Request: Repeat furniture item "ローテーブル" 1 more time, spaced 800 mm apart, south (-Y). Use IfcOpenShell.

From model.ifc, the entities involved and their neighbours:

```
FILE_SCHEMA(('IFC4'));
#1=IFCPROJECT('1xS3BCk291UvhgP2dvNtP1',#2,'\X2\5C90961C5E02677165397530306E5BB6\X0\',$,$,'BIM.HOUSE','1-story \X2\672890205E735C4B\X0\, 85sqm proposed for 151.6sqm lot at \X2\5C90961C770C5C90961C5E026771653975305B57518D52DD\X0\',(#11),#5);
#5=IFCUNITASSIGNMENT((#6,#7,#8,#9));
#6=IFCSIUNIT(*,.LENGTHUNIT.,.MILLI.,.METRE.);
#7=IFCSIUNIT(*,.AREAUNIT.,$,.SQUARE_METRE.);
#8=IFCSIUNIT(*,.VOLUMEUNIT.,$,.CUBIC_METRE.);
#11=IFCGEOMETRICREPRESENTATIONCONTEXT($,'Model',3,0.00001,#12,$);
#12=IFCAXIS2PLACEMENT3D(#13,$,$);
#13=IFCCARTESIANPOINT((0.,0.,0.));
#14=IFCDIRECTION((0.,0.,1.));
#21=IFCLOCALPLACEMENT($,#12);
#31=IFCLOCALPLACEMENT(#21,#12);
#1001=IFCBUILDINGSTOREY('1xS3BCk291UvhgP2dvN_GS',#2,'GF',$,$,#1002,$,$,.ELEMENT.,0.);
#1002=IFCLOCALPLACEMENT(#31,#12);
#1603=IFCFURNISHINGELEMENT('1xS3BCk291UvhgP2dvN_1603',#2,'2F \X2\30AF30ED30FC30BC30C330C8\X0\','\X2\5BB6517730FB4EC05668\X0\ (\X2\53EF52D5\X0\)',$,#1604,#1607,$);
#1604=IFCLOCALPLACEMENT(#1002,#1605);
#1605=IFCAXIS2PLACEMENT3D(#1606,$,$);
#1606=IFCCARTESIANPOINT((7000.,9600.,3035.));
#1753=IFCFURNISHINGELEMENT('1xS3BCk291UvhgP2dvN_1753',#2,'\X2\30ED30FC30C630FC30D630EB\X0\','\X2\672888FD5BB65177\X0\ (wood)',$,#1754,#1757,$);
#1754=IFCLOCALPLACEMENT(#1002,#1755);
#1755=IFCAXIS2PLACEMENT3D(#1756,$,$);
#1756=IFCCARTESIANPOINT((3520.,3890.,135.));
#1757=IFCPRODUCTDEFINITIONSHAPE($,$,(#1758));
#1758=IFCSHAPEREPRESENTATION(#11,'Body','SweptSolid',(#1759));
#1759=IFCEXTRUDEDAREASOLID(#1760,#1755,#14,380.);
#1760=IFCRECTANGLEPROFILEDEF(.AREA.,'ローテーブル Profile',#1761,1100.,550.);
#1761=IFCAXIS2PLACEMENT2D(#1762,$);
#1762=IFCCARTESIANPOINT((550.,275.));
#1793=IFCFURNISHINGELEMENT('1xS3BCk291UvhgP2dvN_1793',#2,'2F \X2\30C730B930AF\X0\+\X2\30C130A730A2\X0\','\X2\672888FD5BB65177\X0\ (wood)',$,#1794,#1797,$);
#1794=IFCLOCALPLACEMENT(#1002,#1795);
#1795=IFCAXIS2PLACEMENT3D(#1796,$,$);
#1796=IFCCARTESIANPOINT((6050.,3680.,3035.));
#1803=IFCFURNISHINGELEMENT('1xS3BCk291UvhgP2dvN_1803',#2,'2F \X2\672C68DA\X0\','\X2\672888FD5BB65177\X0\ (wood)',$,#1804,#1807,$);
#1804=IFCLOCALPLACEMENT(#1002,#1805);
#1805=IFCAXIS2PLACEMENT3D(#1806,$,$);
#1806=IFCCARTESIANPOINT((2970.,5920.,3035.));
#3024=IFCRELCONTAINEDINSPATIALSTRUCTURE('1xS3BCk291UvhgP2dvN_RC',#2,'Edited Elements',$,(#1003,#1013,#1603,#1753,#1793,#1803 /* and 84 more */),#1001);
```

```python
import numpy as np
import ifcopenshell
import ifcopenshell.api.geometry
import ifcopenshell.api.root
import ifcopenshell.util.element
import ifcopenshell.util.placement
import ifcopenshell.util.unit

model = ifcopenshell.open("model.ifc")
unit_scale = ifcopenshell.util.unit.calculate_unit_scale(model)


def reuse_history(source, copy):
    """copy_class also copies each property set's owner history, people and application; keep the originals."""
    for rel in copy.IsDefinedBy:
        if rel.is_a("IfcRelDefinesByProperties") and (history := rel.RelatingPropertyDefinition.OwnerHistory):
            rel.RelatingPropertyDefinition.OwnerHistory = source.OwnerHistory
            ifcopenshell.util.element.remove_deep2(model, history)


source = model.by_id(1753)
base = ifcopenshell.util.placement.get_local_placement(source.ObjectPlacement)
step = np.array([0.0, -1.0, 0.0]) * 0.8 / unit_scale

for i in range(1, 2):
    copy = ifcopenshell.api.root.copy_class(model, product=source)
    copy.Representation = ifcopenshell.util.element.copy_deep(
        model, source.Representation, exclude=["IfcGeometricRepresentationContext", "IfcRepresentationMap"]
    )
    reuse_history(source, copy)
    matrix = base.copy()
    matrix[:3, 3] += i * step
    print("added at", matrix[:3, 3].round(3) + 0.0)
    ifcopenshell.api.geometry.edit_object_placement(model, product=copy, matrix=matrix, is_si=False)

model.write("model_updated.ifc")
```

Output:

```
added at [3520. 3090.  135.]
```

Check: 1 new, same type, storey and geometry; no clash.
